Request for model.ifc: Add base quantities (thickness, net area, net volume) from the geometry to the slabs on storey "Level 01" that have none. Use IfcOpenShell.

First a look at what the model holds.

```python
import ifcopenshell
import ifcopenshell.util.element
import ifcopenshell.util.unit

model = ifcopenshell.open("model.ifc")
print(model.schema)
for unit_type in ("LENGTHUNIT", "AREAUNIT", "VOLUMEUNIT"):
    print(unit_type, ifcopenshell.util.unit.calculate_unit_scale(model, unit_type))
storey = next(s for s in model.by_type("IfcBuildingStorey") if s.Name == "Level 01")
slabs = [e for e in ifcopenshell.util.element.get_decomposition(storey) if e.is_a("IfcSlab")]
for e in sorted(slabs, key=lambda e: e.id()):
    print(e.id(), e.is_a(), e.Name, list(ifcopenshell.util.element.get_psets(e, qtos_only=True)), sep=" | ")
```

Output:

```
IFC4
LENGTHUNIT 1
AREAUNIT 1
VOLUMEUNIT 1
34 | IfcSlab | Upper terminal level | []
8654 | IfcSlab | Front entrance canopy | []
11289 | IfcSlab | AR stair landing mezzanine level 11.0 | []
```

```python
import ifcopenshell
import ifcopenshell.api.pset
import ifcopenshell.geom
import ifcopenshell.util.element
import ifcopenshell.util.shape
import ifcopenshell.util.unit

model = ifcopenshell.open("model.ifc")
unit_scale = ifcopenshell.util.unit.calculate_unit_scale(model)
area_scale = ifcopenshell.util.unit.calculate_unit_scale(model, "AREAUNIT")
volume_scale = ifcopenshell.util.unit.calculate_unit_scale(model, "VOLUMEUNIT")
settings = ifcopenshell.geom.settings()

storey = next(s for s in model.by_type("IfcBuildingStorey") if s.Name == "Level 01")
slabs = [e for e in ifcopenshell.util.element.get_decomposition(storey) if e.is_a("IfcSlab")]

for e in sorted(slabs, key=lambda e: e.id()):
    if ifcopenshell.util.element.get_psets(e, qtos_only=True, should_inherit=False):
        continue
    # Geometry comes back in metres, in the element's own axes.
    shape = ifcopenshell.geom.create_shape(settings, e)
    values = {
        "Width": ifcopenshell.util.shape.get_z(shape.geometry) / unit_scale,
        "NetArea": ifcopenshell.util.shape.get_footprint_area(shape.geometry) / area_scale,
        "NetVolume": ifcopenshell.util.shape.get_volume(shape.geometry) / volume_scale,
    }
    qto = ifcopenshell.api.pset.add_qto(model, product=e, name="Qto_SlabBaseQuantities")
    ifcopenshell.api.pset.edit_qto(model, qto=qto, properties=values)
    print(e.id(), {k: round(v, 3) for k, v in values.items()})

model.write("model_updated.ifc")
```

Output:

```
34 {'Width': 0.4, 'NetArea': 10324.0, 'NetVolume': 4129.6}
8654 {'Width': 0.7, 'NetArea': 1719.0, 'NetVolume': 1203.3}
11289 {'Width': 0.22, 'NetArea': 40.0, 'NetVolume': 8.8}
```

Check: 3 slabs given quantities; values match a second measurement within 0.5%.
